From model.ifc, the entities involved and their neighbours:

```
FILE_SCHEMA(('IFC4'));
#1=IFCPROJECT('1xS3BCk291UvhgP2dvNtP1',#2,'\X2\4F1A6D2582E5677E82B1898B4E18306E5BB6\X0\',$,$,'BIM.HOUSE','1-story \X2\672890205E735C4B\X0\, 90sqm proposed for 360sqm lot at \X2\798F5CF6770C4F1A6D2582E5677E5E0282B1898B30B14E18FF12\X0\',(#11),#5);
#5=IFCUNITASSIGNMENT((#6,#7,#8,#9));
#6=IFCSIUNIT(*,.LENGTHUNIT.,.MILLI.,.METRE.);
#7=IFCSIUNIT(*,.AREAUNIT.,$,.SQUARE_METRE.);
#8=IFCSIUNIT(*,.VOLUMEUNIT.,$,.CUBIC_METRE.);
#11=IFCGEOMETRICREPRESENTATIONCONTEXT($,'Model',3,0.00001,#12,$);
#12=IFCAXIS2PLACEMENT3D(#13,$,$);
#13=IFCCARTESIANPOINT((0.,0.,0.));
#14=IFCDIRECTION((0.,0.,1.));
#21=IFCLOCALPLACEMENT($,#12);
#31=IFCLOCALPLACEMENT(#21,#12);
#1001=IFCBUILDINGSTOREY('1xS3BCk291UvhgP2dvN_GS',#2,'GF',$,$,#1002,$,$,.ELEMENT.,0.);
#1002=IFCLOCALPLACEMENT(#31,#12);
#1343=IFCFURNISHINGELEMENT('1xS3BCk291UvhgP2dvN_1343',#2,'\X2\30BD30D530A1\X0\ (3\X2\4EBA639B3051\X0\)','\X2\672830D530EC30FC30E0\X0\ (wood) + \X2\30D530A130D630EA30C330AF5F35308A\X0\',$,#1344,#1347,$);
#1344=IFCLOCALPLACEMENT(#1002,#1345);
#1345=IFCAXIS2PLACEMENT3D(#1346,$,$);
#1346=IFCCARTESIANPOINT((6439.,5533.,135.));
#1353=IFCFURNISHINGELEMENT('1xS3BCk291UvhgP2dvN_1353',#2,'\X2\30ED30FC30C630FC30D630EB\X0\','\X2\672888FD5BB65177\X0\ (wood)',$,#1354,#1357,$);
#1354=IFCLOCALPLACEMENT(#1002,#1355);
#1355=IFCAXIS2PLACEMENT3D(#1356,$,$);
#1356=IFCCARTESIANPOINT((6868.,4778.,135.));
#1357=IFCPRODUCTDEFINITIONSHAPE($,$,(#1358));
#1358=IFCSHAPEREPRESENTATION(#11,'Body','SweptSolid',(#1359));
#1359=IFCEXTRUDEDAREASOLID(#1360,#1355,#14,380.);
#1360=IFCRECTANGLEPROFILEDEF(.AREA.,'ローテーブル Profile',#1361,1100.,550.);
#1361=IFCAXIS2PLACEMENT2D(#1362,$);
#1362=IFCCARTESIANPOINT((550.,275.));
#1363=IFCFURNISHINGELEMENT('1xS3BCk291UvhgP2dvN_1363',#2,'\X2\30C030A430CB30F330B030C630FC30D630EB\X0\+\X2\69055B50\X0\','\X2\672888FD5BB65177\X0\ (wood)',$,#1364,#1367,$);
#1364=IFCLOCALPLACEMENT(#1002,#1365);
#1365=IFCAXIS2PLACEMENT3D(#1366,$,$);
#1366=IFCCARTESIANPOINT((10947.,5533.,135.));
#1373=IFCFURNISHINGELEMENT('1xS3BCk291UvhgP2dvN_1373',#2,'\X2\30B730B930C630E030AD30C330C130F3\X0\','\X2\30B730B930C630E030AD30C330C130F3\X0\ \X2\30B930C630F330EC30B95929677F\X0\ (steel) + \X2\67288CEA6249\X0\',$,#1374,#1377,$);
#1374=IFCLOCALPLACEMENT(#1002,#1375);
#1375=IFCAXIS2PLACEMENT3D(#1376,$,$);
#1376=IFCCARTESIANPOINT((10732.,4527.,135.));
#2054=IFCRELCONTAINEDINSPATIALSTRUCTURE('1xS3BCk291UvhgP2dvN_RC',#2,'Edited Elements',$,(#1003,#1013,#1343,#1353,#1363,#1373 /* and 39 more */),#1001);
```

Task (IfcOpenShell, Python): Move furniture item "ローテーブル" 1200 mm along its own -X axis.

```python
import ifcopenshell
import ifcopenshell.api.geometry
import ifcopenshell.util.placement
import ifcopenshell.util.unit

model = ifcopenshell.open("model.ifc")
unit_scale = ifcopenshell.util.unit.calculate_unit_scale(model)

item = model.by_id(1353)
matrix = ifcopenshell.util.placement.get_local_placement(item.ObjectPlacement)
matrix[:3, 3] -= matrix[:3, 0] * 1.2 / unit_scale
ifcopenshell.api.geometry.edit_object_placement(model, product=item, matrix=matrix, is_si=False)

print(ifcopenshell.util.placement.get_local_placement(item.ObjectPlacement).round(3) + 0.0)

model.write("model_v2.ifc")
```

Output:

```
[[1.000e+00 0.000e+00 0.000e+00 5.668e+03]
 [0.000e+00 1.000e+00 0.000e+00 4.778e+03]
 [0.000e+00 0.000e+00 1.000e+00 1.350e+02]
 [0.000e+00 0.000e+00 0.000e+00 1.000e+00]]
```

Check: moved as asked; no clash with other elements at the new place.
